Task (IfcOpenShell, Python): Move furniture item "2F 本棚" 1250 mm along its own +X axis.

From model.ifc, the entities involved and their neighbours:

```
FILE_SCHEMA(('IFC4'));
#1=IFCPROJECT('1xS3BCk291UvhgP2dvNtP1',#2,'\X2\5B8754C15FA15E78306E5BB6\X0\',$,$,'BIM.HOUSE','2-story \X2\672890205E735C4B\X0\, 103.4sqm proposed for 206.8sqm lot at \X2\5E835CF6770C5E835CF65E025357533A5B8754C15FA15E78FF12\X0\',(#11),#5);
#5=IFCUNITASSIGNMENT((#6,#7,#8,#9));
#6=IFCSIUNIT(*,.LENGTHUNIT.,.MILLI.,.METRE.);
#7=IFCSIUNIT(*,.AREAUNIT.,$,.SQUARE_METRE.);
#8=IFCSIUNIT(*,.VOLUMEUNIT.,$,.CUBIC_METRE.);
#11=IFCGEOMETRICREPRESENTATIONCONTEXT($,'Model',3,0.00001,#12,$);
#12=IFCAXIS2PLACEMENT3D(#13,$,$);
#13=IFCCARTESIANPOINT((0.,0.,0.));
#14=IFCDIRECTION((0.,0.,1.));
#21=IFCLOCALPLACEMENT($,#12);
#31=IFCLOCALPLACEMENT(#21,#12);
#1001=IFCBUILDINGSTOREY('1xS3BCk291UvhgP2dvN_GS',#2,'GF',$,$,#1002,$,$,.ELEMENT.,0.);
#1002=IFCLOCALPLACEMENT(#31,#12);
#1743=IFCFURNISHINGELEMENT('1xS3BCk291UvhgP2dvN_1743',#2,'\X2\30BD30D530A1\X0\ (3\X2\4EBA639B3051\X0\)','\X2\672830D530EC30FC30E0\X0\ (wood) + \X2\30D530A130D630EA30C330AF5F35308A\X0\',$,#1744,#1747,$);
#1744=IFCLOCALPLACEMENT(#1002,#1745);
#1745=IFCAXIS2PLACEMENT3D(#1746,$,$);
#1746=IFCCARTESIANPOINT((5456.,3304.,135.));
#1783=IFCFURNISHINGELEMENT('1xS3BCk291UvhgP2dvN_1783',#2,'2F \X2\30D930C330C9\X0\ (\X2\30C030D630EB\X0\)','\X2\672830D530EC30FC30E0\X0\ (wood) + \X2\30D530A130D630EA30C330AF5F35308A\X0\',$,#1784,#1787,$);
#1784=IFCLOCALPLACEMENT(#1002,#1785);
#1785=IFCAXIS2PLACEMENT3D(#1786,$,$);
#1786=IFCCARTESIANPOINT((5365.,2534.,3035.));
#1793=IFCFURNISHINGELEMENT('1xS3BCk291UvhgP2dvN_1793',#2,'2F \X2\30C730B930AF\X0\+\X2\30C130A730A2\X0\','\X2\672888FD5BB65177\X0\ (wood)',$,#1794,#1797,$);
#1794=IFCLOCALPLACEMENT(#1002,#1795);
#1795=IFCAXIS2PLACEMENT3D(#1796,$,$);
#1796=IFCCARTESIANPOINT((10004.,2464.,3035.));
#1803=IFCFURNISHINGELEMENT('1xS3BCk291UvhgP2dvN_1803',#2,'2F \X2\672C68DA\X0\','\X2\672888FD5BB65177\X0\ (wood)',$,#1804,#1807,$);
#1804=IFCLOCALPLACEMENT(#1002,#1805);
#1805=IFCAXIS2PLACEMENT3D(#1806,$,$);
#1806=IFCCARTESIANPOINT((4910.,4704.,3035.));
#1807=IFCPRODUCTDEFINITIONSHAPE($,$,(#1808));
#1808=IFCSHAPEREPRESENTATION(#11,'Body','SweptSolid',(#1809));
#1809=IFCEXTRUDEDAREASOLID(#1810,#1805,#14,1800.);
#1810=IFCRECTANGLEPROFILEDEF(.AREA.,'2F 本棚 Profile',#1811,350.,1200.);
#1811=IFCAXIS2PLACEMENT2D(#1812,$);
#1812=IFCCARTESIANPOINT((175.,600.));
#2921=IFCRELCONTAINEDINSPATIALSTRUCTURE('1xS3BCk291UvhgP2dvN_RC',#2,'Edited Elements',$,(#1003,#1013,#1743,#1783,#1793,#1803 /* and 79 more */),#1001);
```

```python
import ifcopenshell
import ifcopenshell.api.geometry
import ifcopenshell.util.placement
import ifcopenshell.util.unit

model = ifcopenshell.open("model.ifc")
unit_scale = ifcopenshell.util.unit.calculate_unit_scale(model)

item = model.by_id(1803)
matrix = ifcopenshell.util.placement.get_local_placement(item.ObjectPlacement)
matrix[:3, 3] += matrix[:3, 0] * 1.25 / unit_scale
ifcopenshell.api.geometry.edit_object_placement(model, product=item, matrix=matrix, is_si=False)

print(ifcopenshell.util.placement.get_local_placement(item.ObjectPlacement).round(3) + 0.0)

model.write("model_rev.ifc")
```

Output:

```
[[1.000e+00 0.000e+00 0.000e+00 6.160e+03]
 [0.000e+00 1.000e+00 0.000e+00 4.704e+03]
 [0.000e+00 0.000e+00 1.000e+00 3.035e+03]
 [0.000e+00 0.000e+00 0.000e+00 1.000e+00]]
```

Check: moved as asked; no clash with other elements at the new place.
